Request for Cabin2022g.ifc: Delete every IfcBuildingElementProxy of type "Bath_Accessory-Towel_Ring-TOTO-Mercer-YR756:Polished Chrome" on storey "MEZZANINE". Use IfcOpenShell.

First a look at what the model holds.

```python
import ifcopenshell
import ifcopenshell.util.element

model = ifcopenshell.open("Cabin2022g.ifc")
print(model.schema)
storey = next(s for s in model.by_type("IfcBuildingStorey") if s.Name == "MEZZANINE")
proxies = [e for e in ifcopenshell.util.element.get_decomposition(storey) if e.is_a("IfcBuildingElementProxy")]
seen = {}
for e in proxies:
    element_type = ifcopenshell.util.element.get_type(e)
    name = element_type.Name if element_type not in (None, e) else None
    seen[name] = seen.get(name, 0) + 1
for name, count in sorted(seen.items(), key=str):
    print(count, "x", name)
```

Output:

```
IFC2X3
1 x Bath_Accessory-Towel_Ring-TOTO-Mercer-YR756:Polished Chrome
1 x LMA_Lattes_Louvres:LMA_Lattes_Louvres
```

```python
import ifcopenshell
import ifcopenshell.api.root
import ifcopenshell.util.element

model = ifcopenshell.open("Cabin2022g.ifc")

storey = next(s for s in model.by_type("IfcBuildingStorey") if s.Name == "MEZZANINE")
proxies = [e for e in ifcopenshell.util.element.get_decomposition(storey) if e.is_a("IfcBuildingElementProxy")]
targets = [e for e in proxies if (t := ifcopenshell.util.element.get_type(e)) not in (None, e) and t.Name == "Bath_Accessory-Towel_Ring-TOTO-Mercer-YR756:Polished Chrome"]

for e in targets:
    ifcopenshell.api.root.remove_product(model, product=e)
print(len(targets), "removed")

model.write("Cabin2022g_edited.ifc")
```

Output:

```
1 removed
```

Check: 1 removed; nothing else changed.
